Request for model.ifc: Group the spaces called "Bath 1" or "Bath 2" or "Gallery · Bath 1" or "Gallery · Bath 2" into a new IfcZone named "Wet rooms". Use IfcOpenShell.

First a look at what the model holds.

```python
import ifcopenshell

model = ifcopenshell.open("model.ifc")
print(model.schema)
seen = {}
for space in model.by_type("IfcSpace"):
    seen[space.Name] = seen.get(space.Name, 0) + 1
for name, count in sorted(seen.items(), key=str):
    print(count, "x", name)
print("zones:", [z.Name for z in model.by_type("IfcZone")][:20])
```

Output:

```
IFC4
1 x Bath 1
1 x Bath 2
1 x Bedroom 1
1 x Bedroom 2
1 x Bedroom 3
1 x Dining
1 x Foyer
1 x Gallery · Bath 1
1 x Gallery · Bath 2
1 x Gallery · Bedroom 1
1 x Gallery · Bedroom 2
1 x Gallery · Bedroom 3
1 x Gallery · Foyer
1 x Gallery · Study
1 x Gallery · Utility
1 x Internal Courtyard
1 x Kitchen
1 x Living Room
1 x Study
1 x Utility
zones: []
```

```python
import ifcopenshell
import ifcopenshell.api.group
import ifcopenshell.api.root

model = ifcopenshell.open("model.ifc")

names = {"Bath 1", "Bath 2", "Gallery · Bath 1", "Gallery · Bath 2"}
spaces = [s for s in model.by_type("IfcSpace") if s.Name in names]

zone = ifcopenshell.api.root.create_entity(model, ifc_class="IfcZone", name="Wet rooms")
ifcopenshell.api.group.assign_group(model, products=spaces, group=zone)
print(len(spaces), "spaces in", zone.Name)

model.write("model_rev.ifc")
```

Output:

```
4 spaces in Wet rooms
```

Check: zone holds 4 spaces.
